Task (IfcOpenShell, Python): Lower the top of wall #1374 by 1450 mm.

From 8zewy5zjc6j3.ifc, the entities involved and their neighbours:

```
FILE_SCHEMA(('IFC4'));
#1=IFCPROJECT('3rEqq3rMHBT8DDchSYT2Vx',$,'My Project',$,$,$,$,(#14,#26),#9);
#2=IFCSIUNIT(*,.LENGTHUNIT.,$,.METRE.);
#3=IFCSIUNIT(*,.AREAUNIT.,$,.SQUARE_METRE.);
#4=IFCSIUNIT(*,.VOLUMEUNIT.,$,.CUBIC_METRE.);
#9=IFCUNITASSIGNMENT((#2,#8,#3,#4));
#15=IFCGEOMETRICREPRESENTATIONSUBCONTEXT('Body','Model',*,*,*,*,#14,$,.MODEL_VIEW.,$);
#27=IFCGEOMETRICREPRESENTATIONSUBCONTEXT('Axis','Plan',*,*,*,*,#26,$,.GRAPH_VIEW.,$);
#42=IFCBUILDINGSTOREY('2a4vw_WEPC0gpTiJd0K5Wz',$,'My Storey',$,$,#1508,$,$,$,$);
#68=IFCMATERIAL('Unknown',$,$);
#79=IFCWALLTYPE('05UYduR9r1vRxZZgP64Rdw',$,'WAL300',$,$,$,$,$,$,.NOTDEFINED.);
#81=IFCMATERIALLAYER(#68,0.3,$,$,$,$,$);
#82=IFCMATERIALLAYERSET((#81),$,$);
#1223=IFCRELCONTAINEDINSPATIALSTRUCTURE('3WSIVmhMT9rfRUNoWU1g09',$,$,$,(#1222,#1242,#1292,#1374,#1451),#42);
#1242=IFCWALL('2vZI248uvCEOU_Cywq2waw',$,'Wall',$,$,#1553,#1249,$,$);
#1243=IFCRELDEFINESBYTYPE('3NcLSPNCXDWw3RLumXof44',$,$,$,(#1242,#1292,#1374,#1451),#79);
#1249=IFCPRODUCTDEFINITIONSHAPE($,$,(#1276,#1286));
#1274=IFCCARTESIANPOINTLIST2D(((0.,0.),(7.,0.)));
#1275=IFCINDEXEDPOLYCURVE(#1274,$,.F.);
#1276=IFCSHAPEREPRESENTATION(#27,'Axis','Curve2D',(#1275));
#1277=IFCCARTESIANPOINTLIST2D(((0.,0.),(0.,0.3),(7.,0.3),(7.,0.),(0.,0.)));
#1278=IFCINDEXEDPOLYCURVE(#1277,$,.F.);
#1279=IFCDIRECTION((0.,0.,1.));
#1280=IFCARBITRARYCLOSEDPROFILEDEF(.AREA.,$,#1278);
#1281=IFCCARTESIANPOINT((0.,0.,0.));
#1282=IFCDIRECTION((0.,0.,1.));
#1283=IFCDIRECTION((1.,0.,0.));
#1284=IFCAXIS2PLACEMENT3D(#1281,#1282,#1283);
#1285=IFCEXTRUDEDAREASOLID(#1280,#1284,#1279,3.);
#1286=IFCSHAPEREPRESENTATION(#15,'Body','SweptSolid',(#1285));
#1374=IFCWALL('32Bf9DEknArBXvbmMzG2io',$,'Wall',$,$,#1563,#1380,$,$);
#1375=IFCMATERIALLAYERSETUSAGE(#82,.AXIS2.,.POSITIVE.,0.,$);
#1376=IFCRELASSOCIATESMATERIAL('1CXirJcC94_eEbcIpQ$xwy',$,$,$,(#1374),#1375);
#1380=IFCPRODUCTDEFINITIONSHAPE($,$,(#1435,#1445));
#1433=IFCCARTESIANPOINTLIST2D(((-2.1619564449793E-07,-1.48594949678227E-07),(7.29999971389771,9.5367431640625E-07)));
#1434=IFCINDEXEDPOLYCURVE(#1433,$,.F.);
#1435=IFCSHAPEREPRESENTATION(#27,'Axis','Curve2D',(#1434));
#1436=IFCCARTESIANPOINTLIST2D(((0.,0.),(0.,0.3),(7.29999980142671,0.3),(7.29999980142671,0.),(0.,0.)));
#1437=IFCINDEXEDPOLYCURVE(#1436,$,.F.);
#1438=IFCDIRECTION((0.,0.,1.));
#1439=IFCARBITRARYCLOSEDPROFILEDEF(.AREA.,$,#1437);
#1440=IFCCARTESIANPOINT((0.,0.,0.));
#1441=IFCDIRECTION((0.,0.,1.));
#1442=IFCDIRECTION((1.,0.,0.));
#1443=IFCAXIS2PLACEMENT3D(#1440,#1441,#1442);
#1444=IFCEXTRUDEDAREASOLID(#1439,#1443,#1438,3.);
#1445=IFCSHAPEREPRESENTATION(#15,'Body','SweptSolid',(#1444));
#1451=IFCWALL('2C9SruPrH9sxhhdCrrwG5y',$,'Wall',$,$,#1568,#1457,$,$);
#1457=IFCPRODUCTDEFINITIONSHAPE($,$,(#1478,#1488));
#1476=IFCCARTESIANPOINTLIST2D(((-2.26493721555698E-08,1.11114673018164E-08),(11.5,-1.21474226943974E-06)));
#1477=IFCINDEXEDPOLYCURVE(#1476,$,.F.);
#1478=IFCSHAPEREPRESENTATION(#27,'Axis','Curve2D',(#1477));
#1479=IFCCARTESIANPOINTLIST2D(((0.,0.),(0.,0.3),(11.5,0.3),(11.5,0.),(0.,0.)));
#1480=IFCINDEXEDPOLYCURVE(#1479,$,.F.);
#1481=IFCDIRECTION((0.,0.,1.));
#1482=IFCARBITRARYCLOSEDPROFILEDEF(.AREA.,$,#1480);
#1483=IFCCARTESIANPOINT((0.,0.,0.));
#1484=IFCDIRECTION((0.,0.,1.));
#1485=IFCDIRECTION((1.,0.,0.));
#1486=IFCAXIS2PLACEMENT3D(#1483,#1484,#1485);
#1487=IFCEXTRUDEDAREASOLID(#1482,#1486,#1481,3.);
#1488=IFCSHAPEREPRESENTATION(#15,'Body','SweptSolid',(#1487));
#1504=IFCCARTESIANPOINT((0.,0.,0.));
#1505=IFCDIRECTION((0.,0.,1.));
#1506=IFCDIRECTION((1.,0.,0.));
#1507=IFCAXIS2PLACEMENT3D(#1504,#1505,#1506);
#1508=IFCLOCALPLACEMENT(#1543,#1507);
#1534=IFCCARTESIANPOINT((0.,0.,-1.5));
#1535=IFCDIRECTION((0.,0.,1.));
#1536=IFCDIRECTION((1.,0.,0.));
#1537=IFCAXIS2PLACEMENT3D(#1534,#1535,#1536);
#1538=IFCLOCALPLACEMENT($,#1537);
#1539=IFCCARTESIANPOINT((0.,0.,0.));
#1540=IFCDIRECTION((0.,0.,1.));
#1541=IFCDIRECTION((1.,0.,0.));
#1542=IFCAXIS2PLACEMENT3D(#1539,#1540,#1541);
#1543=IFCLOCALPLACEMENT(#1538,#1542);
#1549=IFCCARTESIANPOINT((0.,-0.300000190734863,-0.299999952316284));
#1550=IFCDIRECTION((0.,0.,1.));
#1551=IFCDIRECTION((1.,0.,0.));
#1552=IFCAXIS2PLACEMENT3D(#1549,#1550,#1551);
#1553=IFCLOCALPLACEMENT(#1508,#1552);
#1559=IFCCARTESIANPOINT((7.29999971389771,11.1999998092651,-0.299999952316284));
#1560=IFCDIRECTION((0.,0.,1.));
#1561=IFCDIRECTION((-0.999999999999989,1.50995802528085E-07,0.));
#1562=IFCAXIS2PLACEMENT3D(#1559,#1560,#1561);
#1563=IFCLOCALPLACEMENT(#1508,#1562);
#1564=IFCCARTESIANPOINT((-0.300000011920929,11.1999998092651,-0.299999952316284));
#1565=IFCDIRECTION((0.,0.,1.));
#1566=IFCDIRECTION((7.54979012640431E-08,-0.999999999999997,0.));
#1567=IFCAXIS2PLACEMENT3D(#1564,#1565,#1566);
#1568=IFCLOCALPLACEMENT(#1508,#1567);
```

```python
import ifcopenshell
import ifcopenshell.geom
import ifcopenshell.util.representation
import ifcopenshell.util.shape

model = ifcopenshell.open("8zewy5zjc6j3.ifc")
settings = ifcopenshell.geom.settings()


def volume(element):
    """Net volume in cubic metres, openings subtracted."""
    shape = ifcopenshell.geom.create_shape(settings, element)
    return ifcopenshell.util.shape.get_volume(shape.geometry)


wall = model.by_guid("32Bf9DEknArBXvbmMzG2io")
before = volume(wall)

body = ifcopenshell.util.representation.get_representation(wall, "Model", "Body")
solid = body.Items[0]
old_height = solid.Depth
solid.Depth -= 1.45
after = volume(wall)

print(f"height {old_height:g} -> {solid.Depth:g}, volume {before:.3f} -> {after:.3f} m3")

model.write("8zewy5zjc6j3_rev.ifc")
```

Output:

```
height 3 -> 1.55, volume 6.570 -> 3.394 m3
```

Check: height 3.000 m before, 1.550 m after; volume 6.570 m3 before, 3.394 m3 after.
